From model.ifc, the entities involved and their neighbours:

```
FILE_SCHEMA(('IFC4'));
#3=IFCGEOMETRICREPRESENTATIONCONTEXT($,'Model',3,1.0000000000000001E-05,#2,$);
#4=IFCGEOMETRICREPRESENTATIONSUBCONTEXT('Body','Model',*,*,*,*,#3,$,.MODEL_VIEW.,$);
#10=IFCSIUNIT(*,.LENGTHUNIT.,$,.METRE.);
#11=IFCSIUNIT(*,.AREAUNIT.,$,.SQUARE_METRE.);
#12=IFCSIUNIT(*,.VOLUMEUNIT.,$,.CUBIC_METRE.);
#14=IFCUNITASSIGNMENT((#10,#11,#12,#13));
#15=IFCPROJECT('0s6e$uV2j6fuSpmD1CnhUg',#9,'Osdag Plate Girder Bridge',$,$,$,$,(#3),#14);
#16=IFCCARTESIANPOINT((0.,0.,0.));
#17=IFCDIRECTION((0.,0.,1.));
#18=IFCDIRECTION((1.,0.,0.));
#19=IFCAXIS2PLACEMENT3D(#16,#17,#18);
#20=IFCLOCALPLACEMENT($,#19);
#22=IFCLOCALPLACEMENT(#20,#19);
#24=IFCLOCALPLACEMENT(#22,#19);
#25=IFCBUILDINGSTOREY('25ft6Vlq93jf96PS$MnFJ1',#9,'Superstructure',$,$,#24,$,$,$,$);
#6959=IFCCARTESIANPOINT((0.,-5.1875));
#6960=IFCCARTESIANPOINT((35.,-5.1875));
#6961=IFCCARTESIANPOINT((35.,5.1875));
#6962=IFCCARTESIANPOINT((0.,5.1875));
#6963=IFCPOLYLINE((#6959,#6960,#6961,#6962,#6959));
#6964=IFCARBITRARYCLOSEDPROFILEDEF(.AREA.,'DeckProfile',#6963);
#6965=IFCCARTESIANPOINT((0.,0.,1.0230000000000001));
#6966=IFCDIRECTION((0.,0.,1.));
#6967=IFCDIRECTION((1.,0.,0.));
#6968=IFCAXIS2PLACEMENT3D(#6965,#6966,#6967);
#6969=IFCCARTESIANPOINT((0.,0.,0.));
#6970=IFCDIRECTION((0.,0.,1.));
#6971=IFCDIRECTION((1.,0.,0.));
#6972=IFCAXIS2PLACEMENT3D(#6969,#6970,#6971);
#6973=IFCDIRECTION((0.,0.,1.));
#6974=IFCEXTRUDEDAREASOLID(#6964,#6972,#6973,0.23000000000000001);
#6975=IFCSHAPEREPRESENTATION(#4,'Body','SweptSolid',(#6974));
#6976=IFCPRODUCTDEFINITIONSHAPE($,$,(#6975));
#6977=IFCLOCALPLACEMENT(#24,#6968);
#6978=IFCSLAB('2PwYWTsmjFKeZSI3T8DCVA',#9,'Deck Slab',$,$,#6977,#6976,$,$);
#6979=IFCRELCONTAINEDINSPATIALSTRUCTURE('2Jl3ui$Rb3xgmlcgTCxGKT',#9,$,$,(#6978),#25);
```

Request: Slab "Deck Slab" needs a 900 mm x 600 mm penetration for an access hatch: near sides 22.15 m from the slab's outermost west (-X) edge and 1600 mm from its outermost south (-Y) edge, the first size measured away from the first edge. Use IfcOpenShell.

```python
import numpy as np
import ifcopenshell
import ifcopenshell.api.feature
import ifcopenshell.api.geometry
import ifcopenshell.api.root
import ifcopenshell.geom
import ifcopenshell.util.placement
import ifcopenshell.util.representation
import ifcopenshell.util.shape
import ifcopenshell.util.unit

model = ifcopenshell.open("model.ifc")
unit_scale = ifcopenshell.util.unit.calculate_unit_scale(model)
settings = ifcopenshell.geom.settings()


def volume(element):
    """Net volume in cubic metres, openings subtracted."""
    shape = ifcopenshell.geom.create_shape(settings, element)
    return ifcopenshell.util.shape.get_volume(shape.geometry)


slab = model.by_guid("2PwYWTsmjFKeZSI3T8DCVA")
before = volume(slab)

# Extent in the slab's own axes, in metres. The edges named are its -X and -Y sides.
slab_shape = ifcopenshell.geom.create_shape(settings, slab)
vertices = ifcopenshell.util.shape.get_vertices(slab_shape.geometry)
x_min, y_min, bottom = vertices.min(axis=0)
top = vertices[:, 2].max()

opening = ifcopenshell.api.root.create_entity(model, ifc_class="IfcOpeningElement", name="Access hatch opening", predefined_type="OPENING")
context = ifcopenshell.util.representation.get_context(model, "Model", "Body", "MODEL_VIEW")
width, depth = 0.9, 0.6
outline = [(0.0, 0.0), (width, 0.0), (width, depth), (0.0, depth), (0.0, 0.0)]
# Overshoot both faces by 50 mm so the cut is clean.
shape = ifcopenshell.api.geometry.add_slab_representation(
    model, context=context, depth=top - bottom + 0.1, polyline=outline
)
ifcopenshell.api.geometry.assign_representation(model, product=opening, representation=shape)

matrix = ifcopenshell.util.placement.get_local_placement(slab.ObjectPlacement)
matrix[:, 3] = matrix @ np.append(np.array([x_min + 22.15, y_min + 1.6, bottom - 0.05]) / unit_scale, 1.0)
ifcopenshell.api.geometry.edit_object_placement(model, product=opening, matrix=matrix, is_si=False)
ifcopenshell.api.feature.add_feature(model, feature=opening, element=slab)

after = volume(slab)

print(f"slab volume {before:.3f} -> {after:.3f} m3")

model.write("model_rev.ifc")
```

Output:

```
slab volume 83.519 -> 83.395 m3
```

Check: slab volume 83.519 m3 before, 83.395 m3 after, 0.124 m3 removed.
